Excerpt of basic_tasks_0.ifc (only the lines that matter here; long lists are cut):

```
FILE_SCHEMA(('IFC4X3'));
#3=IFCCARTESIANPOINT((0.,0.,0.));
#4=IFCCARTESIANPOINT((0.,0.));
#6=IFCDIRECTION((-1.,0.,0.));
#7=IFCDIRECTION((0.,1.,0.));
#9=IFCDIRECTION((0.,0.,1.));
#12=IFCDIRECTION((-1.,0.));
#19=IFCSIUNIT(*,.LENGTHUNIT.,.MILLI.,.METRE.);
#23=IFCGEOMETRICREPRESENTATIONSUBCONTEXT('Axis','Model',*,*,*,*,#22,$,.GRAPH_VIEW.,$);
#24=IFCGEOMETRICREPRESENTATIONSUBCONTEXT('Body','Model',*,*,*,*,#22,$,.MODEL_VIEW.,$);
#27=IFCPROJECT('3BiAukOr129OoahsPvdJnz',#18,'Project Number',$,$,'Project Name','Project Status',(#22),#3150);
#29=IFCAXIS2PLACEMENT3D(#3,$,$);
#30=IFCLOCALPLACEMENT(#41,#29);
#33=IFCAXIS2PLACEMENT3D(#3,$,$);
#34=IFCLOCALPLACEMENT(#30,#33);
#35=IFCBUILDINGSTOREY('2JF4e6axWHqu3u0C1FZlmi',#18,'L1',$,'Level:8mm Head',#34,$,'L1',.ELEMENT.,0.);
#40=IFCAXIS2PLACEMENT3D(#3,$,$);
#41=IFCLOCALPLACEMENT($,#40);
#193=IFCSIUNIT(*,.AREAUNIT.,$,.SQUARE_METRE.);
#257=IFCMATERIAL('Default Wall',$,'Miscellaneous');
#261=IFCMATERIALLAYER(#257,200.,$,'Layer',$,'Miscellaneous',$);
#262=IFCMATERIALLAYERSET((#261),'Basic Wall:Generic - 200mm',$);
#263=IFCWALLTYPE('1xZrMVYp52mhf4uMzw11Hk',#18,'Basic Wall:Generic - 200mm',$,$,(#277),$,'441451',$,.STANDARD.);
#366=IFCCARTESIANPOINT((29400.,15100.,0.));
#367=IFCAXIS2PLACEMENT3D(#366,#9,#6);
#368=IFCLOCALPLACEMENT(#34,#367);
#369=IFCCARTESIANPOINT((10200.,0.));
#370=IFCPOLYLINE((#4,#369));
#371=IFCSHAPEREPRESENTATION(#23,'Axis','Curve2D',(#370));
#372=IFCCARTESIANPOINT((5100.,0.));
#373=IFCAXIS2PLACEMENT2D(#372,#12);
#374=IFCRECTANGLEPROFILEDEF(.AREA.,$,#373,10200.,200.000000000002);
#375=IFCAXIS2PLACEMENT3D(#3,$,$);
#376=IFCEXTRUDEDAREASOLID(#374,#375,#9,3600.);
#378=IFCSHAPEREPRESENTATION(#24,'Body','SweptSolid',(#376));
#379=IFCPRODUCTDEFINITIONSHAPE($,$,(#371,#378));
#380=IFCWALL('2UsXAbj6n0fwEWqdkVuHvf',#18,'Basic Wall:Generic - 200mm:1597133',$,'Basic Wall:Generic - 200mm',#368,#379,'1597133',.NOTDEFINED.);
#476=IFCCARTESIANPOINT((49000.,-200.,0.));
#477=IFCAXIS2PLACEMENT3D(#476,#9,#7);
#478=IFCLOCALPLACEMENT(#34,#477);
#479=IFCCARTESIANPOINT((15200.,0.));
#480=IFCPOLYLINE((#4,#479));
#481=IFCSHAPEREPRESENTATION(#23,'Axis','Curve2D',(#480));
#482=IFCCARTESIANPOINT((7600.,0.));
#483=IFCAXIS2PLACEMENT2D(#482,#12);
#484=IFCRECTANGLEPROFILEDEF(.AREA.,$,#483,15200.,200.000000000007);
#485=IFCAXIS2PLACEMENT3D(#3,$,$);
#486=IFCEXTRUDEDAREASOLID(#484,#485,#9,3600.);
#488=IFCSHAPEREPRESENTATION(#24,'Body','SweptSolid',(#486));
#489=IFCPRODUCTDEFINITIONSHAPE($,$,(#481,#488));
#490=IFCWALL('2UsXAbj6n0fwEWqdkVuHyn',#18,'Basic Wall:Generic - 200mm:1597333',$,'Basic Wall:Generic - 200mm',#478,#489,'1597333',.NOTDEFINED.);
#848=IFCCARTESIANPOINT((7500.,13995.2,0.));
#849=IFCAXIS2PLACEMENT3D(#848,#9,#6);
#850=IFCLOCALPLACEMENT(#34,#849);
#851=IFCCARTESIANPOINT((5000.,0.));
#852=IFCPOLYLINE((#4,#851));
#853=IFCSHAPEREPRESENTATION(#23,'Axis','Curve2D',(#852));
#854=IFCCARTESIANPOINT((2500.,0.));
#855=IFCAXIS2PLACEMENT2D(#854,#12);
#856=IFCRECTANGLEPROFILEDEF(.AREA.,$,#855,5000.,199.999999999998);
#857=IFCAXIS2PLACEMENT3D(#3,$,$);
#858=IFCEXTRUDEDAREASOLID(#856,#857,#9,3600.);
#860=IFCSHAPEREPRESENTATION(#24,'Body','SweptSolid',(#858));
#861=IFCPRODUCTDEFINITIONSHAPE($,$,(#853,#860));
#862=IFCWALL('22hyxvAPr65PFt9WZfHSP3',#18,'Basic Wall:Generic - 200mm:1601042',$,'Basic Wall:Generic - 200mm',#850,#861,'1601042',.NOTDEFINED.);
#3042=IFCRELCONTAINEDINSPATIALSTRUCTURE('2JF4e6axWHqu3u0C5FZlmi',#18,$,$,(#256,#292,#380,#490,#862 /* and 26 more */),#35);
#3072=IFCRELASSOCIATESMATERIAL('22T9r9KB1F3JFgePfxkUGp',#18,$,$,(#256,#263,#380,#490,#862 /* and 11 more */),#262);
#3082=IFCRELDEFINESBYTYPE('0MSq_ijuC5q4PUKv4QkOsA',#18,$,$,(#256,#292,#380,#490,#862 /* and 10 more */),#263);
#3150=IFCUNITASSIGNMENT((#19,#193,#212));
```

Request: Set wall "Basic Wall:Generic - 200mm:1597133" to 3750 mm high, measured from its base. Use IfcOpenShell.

```python
import ifcopenshell
import ifcopenshell.geom
import ifcopenshell.util.representation
import ifcopenshell.util.shape

model = ifcopenshell.open("basic_tasks_0.ifc")
settings = ifcopenshell.geom.settings()


def volume(element):
    """Net volume in cubic metres, openings subtracted."""
    shape = ifcopenshell.geom.create_shape(settings, element)
    return ifcopenshell.util.shape.get_volume(shape.geometry)


wall = model.by_guid("2UsXAbj6n0fwEWqdkVuHvf")
before = volume(wall)

body = ifcopenshell.util.representation.get_representation(wall, "Model", "Body")
solid = body.Items[0]
old_height = solid.Depth
solid.Depth = 3750.0
after = volume(wall)

print(f"height {old_height:g} -> {solid.Depth:g}, volume {before:.3f} -> {after:.3f} m3")

model.write("basic_tasks_0_edited.ifc")
```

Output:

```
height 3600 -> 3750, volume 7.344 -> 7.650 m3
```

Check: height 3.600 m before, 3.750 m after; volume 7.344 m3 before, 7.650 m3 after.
